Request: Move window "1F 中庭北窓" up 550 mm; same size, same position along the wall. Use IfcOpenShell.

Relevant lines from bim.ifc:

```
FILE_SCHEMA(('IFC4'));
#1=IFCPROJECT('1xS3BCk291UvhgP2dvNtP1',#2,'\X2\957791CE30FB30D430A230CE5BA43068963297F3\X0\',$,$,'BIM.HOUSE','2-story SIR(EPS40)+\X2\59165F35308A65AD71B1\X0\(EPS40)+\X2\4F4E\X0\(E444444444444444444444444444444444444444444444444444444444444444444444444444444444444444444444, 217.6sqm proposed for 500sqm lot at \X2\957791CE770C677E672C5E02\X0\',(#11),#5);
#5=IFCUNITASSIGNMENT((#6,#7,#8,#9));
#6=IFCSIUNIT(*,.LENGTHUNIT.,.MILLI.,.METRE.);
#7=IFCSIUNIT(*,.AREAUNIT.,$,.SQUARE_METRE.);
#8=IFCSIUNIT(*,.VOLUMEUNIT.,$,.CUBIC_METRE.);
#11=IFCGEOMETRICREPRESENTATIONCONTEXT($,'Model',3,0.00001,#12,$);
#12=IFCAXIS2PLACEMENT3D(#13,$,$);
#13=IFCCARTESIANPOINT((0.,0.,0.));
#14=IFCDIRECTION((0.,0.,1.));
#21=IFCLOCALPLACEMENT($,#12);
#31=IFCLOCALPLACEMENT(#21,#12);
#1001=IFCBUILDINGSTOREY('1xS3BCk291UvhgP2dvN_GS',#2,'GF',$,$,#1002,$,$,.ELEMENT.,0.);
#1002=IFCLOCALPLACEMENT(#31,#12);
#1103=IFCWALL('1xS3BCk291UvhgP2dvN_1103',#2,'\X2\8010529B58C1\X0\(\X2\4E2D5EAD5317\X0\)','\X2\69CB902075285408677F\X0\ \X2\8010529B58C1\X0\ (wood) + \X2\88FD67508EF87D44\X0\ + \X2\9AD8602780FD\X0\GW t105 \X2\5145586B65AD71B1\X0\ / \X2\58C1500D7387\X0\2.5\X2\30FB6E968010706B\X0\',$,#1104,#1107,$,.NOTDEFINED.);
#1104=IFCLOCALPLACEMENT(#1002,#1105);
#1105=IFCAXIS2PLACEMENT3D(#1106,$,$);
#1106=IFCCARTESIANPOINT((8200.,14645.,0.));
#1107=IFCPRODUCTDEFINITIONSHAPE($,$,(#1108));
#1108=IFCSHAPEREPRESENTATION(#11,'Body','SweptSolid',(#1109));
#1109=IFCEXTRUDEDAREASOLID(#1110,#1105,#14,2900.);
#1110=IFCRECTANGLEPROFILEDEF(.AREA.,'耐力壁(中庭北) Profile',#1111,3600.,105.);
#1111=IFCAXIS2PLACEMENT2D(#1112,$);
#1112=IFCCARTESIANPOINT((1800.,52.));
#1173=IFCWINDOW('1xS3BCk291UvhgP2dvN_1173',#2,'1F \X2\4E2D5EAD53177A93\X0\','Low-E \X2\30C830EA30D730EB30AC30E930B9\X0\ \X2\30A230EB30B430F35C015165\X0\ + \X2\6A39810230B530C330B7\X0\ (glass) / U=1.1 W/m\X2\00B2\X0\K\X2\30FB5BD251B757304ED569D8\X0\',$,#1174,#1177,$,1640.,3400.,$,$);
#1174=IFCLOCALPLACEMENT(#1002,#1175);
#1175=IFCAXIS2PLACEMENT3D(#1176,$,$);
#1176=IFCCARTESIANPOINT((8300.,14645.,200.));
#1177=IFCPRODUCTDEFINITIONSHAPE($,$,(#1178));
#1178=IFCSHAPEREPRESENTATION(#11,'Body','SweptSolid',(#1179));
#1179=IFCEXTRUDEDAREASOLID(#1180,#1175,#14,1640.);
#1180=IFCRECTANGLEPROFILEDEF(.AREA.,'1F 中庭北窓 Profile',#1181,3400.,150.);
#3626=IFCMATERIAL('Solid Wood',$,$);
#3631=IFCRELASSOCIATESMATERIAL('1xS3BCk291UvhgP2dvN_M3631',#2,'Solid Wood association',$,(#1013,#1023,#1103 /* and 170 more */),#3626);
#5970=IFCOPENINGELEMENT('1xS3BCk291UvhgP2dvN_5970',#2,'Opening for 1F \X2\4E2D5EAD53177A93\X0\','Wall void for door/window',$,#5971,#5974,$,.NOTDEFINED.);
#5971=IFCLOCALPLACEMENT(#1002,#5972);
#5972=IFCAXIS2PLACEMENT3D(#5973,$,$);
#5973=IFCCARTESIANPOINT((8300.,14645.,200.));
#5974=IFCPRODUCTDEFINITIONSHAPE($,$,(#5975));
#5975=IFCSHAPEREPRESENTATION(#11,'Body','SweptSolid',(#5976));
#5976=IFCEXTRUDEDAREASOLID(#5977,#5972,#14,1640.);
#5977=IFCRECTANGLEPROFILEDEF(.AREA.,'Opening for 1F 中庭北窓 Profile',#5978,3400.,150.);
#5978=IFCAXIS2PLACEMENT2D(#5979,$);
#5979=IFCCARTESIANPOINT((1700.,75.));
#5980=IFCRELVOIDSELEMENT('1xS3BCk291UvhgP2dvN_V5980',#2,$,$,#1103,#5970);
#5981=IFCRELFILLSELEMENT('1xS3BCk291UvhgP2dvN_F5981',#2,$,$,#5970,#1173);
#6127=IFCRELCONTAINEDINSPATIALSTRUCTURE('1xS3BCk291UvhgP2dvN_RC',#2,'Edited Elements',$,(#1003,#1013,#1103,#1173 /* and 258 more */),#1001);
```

```python
import numpy as np
import ifcopenshell
import ifcopenshell.api.geometry
import ifcopenshell.util.placement
import ifcopenshell.util.unit

model = ifcopenshell.open("bim.ifc")
unit_scale = ifcopenshell.util.unit.calculate_unit_scale(model)

window = model.by_guid("1xS3BCk291UvhgP2dvN_1173")
opening = window.FillsVoids[0].RelatingOpeningElement
dz = 550.0

shift = np.array([0.0, 0.0, dz])
# The window is not placed relative to its opening, so move both.
for product in (opening, window):
    matrix = ifcopenshell.util.placement.get_local_placement(product.ObjectPlacement)
    matrix[:3, 3] += shift
    ifcopenshell.api.geometry.edit_object_placement(model, product=product, matrix=matrix, is_si=False)

print(f"moved by {dz * unit_scale:+.3f} m")

model.write("bim_rev.ifc")
```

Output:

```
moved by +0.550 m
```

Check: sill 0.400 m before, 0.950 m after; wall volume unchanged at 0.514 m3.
